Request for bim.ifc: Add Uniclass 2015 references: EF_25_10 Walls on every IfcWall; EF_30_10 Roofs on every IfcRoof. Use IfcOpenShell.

First a look at what the model holds.

```python
import ifcopenshell

model = ifcopenshell.open("bim.ifc")
print(model.schema)
print("classifications:", [c.Name for c in model.by_type("IfcClassification")])
for ifc_class in ("IfcDoor", "IfcRoof", "IfcStair", "IfcWall", "IfcWindow"):
    print(ifc_class, len(model.by_type(ifc_class)))
```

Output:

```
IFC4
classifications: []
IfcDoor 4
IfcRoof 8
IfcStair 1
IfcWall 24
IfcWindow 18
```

```python
import ifcopenshell
import ifcopenshell.api.classification

model = ifcopenshell.open("bim.ifc")

system = ifcopenshell.api.classification.add_classification(model, classification="Uniclass 2015")

codes = {
    "IfcWall": ("EF_25_10", "Walls"),
    "IfcRoof": ("EF_30_10", "Roofs"),
}
for ifc_class, (code, name) in codes.items():
    products = model.by_type(ifc_class)
    ifcopenshell.api.classification.add_reference(
        model, products=products, classification=system, identification=code, name=name
    )
    print(code, len(products))

model.write("bim-out.ifc")
```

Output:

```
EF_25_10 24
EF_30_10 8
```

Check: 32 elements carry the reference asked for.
